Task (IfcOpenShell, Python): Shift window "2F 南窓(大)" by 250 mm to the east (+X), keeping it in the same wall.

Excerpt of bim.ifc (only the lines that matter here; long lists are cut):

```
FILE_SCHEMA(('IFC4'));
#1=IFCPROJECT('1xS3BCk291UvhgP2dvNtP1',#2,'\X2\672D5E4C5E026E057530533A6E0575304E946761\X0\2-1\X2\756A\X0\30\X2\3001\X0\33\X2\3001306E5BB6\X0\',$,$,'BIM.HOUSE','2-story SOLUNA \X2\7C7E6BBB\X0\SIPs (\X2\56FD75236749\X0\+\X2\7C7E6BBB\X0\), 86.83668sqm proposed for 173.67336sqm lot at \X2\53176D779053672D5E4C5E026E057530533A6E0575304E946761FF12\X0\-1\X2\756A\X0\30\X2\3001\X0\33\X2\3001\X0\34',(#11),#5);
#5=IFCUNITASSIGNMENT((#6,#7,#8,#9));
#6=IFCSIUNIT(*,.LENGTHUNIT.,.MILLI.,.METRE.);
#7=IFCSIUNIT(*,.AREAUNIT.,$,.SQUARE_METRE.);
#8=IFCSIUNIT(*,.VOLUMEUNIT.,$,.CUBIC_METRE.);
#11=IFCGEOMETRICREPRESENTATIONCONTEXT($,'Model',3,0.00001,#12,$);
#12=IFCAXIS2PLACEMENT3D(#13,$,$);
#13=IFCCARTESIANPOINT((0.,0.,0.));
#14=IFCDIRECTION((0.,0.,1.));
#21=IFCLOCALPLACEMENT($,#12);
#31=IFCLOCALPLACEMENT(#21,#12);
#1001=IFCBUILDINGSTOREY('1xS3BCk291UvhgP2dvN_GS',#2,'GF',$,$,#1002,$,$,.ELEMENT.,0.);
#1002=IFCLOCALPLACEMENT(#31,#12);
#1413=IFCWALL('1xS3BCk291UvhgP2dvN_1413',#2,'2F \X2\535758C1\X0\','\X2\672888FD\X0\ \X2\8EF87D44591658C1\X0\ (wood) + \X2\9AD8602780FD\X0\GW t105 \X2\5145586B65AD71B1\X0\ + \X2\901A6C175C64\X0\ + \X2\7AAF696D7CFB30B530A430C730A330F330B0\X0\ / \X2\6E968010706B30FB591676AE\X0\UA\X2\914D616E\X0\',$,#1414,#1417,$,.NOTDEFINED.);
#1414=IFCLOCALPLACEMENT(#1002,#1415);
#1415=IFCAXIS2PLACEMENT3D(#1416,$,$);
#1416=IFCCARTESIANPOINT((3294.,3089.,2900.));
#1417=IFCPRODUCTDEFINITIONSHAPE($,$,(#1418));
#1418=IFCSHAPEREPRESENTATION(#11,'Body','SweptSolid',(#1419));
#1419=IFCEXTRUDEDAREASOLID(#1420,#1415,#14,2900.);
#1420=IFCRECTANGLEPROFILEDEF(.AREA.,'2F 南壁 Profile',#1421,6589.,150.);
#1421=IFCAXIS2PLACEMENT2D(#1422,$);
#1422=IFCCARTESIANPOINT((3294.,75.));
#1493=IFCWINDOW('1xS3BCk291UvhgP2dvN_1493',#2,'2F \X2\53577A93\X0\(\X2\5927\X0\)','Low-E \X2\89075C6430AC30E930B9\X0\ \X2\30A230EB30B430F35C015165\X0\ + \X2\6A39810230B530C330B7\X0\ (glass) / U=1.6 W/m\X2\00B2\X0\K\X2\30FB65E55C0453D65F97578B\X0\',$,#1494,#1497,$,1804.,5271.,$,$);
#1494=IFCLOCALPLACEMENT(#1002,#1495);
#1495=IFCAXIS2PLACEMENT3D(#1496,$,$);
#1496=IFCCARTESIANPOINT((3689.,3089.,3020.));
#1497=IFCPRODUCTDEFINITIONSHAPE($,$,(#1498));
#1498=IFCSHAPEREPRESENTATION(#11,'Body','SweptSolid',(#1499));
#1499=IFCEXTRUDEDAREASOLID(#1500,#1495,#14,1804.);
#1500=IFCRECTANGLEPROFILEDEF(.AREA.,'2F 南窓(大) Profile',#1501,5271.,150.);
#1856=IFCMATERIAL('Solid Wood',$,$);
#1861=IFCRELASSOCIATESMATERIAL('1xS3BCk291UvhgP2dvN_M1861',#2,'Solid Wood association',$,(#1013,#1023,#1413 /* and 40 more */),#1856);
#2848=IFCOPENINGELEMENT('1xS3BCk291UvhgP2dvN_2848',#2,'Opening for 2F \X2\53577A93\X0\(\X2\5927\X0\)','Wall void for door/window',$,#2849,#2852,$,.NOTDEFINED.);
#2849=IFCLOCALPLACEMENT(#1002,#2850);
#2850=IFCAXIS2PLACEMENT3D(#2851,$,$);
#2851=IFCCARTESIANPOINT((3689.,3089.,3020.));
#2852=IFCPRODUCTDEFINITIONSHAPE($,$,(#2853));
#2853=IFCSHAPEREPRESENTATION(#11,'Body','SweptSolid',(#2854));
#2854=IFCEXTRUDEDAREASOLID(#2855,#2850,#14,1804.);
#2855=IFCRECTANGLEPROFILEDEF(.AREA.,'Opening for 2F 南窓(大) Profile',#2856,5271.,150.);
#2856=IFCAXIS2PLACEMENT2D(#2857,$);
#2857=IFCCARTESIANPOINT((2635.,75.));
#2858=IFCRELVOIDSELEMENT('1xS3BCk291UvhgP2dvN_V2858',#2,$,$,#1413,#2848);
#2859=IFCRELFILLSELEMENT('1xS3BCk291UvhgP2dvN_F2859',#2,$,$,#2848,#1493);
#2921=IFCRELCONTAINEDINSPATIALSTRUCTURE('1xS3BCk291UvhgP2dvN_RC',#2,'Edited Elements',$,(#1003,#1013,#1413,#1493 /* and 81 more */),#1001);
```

```python
import ifcopenshell
import ifcopenshell.api.geometry
import ifcopenshell.util.placement
import ifcopenshell.util.unit

model = ifcopenshell.open("bim.ifc")
unit_scale = ifcopenshell.util.unit.calculate_unit_scale(model)

window = model.by_guid("1xS3BCk291UvhgP2dvN_1493")
opening = window.FillsVoids[0].RelatingOpeningElement
wall = opening.VoidsElements[0].RelatingBuildingElement

wall_matrix = ifcopenshell.util.placement.get_local_placement(wall.ObjectPlacement)
shift = wall_matrix[:3, 0] * 0.25 / unit_scale
before = ifcopenshell.util.placement.get_local_placement(window.ObjectPlacement)[:3, 3].copy()

# The window is not placed relative to its opening, so move both.
for product in (opening, window):
    matrix = ifcopenshell.util.placement.get_local_placement(product.ObjectPlacement)
    matrix[:3, 3] += shift
    ifcopenshell.api.geometry.edit_object_placement(model, product=product, matrix=matrix, is_si=False)

after = ifcopenshell.util.placement.get_local_placement(window.ObjectPlacement)[:3, 3]
print("window moved by", (after - before).round(3) + 0.0)

model.write("bim_edited.ifc")
```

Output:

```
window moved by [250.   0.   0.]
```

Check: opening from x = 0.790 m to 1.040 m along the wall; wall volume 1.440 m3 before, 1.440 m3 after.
